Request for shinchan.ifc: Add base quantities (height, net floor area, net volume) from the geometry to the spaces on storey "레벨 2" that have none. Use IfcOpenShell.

First a look at what the model holds.

```python
import ifcopenshell
import ifcopenshell.util.element
import ifcopenshell.util.unit

model = ifcopenshell.open("shinchan.ifc")
print(model.schema)
for unit_type in ("LENGTHUNIT", "AREAUNIT", "VOLUMEUNIT"):
    print(unit_type, ifcopenshell.util.unit.calculate_unit_scale(model, unit_type))
storey = next(s for s in model.by_type("IfcBuildingStorey") if s.Name == "레벨 2")
spaces = [e for e in ifcopenshell.util.element.get_decomposition(storey) if e.is_a("IfcSpace")]
for e in sorted(spaces, key=lambda e: e.id()):
    print(e.id(), e.is_a(), e.Name, list(ifcopenshell.util.element.get_psets(e, qtos_only=True)), sep=" | ")
```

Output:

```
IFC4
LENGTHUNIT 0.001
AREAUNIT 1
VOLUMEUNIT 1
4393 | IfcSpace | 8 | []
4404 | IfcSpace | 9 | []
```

```python
import ifcopenshell
import ifcopenshell.api.pset
import ifcopenshell.geom
import ifcopenshell.util.element
import ifcopenshell.util.shape
import ifcopenshell.util.unit

model = ifcopenshell.open("shinchan.ifc")
unit_scale = ifcopenshell.util.unit.calculate_unit_scale(model)
area_scale = ifcopenshell.util.unit.calculate_unit_scale(model, "AREAUNIT")
volume_scale = ifcopenshell.util.unit.calculate_unit_scale(model, "VOLUMEUNIT")
settings = ifcopenshell.geom.settings()

storey = next(s for s in model.by_type("IfcBuildingStorey") if s.Name == "레벨 2")
spaces = [e for e in ifcopenshell.util.element.get_decomposition(storey) if e.is_a("IfcSpace")]

for e in sorted(spaces, key=lambda e: e.id()):
    if ifcopenshell.util.element.get_psets(e, qtos_only=True, should_inherit=False):
        continue
    # Geometry comes back in metres, in the element's own axes.
    shape = ifcopenshell.geom.create_shape(settings, e)
    values = {
        "Height": ifcopenshell.util.shape.get_z(shape.geometry) / unit_scale,
        "NetFloorArea": ifcopenshell.util.shape.get_footprint_area(shape.geometry) / area_scale,
        "NetVolume": ifcopenshell.util.shape.get_volume(shape.geometry) / volume_scale,
    }
    qto = ifcopenshell.api.pset.add_qto(model, product=e, name="Qto_SpaceBaseQuantities")
    ifcopenshell.api.pset.edit_qto(model, qto=qto, properties=values)
    print(e.id(), {k: round(v, 3) for k, v in values.items()})

model.write("shinchan_updated.ifc")
```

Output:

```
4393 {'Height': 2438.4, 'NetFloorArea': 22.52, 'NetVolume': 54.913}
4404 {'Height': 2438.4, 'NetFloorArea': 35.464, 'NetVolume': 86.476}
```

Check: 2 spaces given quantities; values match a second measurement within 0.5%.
